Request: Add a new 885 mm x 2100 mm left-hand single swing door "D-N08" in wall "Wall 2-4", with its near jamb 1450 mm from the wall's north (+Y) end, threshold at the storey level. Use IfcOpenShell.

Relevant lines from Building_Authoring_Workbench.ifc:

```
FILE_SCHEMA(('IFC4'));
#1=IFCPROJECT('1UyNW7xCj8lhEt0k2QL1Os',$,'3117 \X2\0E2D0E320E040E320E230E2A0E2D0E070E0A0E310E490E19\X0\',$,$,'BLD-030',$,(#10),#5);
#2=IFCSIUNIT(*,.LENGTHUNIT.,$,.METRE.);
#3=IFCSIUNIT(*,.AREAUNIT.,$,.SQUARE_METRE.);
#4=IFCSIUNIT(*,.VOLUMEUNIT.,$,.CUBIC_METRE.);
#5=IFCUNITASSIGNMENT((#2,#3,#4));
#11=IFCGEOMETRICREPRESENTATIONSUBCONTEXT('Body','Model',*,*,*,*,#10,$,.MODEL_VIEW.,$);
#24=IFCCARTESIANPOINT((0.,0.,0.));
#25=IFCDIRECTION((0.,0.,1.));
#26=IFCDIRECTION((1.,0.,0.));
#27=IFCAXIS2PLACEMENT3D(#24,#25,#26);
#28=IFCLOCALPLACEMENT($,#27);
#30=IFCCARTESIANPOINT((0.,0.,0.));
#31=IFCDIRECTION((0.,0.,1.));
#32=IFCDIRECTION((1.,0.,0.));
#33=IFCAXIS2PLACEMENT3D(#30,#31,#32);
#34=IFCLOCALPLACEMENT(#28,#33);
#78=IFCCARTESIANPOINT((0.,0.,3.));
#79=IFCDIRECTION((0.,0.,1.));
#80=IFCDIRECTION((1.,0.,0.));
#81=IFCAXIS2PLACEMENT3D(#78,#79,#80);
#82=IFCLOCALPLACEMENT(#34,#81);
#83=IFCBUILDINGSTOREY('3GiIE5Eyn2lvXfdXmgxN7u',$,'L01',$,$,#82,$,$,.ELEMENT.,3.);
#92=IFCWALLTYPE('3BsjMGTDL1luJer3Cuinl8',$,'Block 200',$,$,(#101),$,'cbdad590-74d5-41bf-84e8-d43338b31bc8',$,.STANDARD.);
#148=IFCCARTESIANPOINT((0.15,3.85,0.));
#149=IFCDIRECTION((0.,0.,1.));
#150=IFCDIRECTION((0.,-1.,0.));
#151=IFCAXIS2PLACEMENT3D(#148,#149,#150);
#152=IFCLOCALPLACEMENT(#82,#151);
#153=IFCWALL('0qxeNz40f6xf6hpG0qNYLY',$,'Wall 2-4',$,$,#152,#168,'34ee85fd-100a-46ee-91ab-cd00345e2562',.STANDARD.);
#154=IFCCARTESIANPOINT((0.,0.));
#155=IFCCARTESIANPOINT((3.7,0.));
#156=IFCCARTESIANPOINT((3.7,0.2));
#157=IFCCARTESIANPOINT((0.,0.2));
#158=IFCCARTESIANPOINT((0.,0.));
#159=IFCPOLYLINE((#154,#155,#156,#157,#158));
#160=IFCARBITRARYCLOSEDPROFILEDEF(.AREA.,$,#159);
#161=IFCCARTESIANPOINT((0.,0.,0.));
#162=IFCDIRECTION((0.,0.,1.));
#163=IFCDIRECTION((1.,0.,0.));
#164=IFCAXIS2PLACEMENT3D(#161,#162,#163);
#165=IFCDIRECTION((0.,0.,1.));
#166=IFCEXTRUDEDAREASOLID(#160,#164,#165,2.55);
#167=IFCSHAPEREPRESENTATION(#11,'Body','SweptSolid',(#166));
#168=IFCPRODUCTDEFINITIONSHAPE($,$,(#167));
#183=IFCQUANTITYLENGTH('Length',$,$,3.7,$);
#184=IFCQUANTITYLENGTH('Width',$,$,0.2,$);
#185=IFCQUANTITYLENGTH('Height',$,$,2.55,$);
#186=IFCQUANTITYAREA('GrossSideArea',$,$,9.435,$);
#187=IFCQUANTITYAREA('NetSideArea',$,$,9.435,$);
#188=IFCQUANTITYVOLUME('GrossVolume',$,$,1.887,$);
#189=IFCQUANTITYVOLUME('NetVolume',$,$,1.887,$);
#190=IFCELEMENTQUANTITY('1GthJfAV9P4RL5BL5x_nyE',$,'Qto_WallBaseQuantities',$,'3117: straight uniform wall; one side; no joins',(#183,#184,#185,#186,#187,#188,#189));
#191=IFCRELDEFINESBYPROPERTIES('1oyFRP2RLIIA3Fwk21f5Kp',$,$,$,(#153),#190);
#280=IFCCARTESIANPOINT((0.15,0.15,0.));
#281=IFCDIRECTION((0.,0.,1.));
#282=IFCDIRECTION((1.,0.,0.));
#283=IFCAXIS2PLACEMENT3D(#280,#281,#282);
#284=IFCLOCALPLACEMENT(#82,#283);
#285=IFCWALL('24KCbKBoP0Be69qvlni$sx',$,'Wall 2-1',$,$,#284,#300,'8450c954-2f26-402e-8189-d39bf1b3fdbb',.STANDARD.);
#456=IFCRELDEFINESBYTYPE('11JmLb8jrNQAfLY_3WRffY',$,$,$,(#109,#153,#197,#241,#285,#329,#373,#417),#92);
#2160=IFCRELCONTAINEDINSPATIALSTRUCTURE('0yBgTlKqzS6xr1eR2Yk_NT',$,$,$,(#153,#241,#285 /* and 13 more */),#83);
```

```python
import numpy as np
import ifcopenshell
import ifcopenshell.api.feature
import ifcopenshell.api.geometry
import ifcopenshell.api.pset
import ifcopenshell.api.root
import ifcopenshell.api.spatial
import ifcopenshell.geom
import ifcopenshell.util.element
import ifcopenshell.util.placement
import ifcopenshell.util.representation
import ifcopenshell.util.shape
import ifcopenshell.util.unit

model = ifcopenshell.open("Building_Authoring_Workbench.ifc")
unit_scale = ifcopenshell.util.unit.calculate_unit_scale(model)
area_scale = ifcopenshell.util.unit.calculate_unit_scale(model, "AREAUNIT")
volume_scale = ifcopenshell.util.unit.calculate_unit_scale(model, "VOLUMEUNIT")
settings = ifcopenshell.geom.settings()


def volume(element):
    """Net volume in cubic metres, openings subtracted."""
    shape = ifcopenshell.geom.create_shape(settings, element)
    return ifcopenshell.util.shape.get_volume(shape.geometry)


wall = model.by_guid("0qxeNz40f6xf6hpG0qNYLY")
storey = ifcopenshell.util.element.get_container(wall, ifc_class="IfcBuildingStorey")
context = ifcopenshell.util.representation.get_context(model, "Model", "Body", "MODEL_VIEW")
before = volume(wall)

width, height, from_end, sill = 0.885, 2.1, 1.45, 0.0  # metres

# The wall runs along its own X axis, and the end named is its -X end.
wall_shape = ifcopenshell.geom.create_shape(settings, wall)
x, y, z = ifcopenshell.util.shape.get_vertices(wall_shape.geometry).T
start = x.min() + from_end
face, thickness = float(y.min()), float(y.max() - y.min())
wall_matrix = ifcopenshell.util.placement.get_local_placement(wall.ObjectPlacement)
level = ifcopenshell.util.placement.get_local_placement(storey.ObjectPlacement)[2, 3]


def in_wall(x, y):
    """Placement at x, y metres in the wall's axes, at sill height."""
    matrix = wall_matrix.copy()
    matrix[:, 3] = wall_matrix @ np.array([x / unit_scale, y / unit_scale, 0.0, 1.0])
    matrix[2, 3] = level + sill / unit_scale
    return matrix


# Opening: a box that overshoots both wall faces by 50 mm.
opening = ifcopenshell.api.root.create_entity(model, ifc_class="IfcOpeningElement", predefined_type="OPENING")
box = ifcopenshell.api.geometry.add_wall_representation(
    model, context=context, length=width, height=height, thickness=thickness + 0.1
)
ifcopenshell.api.geometry.assign_representation(model, product=opening, representation=box)
ifcopenshell.api.geometry.edit_object_placement(model, product=opening, matrix=in_wall(start, face - 0.05), is_si=False)
ifcopenshell.api.feature.add_feature(model, feature=opening, element=wall)

door = ifcopenshell.api.root.create_entity(model, ifc_class="IfcDoor", name="D-N08", predefined_type="DOOR")
door.OverallWidth, door.OverallHeight = width / unit_scale, height / unit_scale
door.OperationType = "SINGLE_SWING_LEFT"
body = ifcopenshell.api.geometry.add_door_representation(
    model,
    context=context,
    overall_width=door.OverallWidth,
    overall_height=door.OverallHeight,
    operation_type="SINGLE_SWING_LEFT",
    lining_properties={"LiningDepth": thickness / unit_scale, "ThresholdDepth": thickness / unit_scale},
)
ifcopenshell.api.geometry.assign_representation(model, product=door, representation=body)
ifcopenshell.api.spatial.assign_container(model, products=[door], relating_structure=storey)
ifcopenshell.api.feature.add_filling(model, opening=opening, element=door)

# The lining spans the wall, so the door starts at the wall face.
ifcopenshell.api.geometry.edit_object_placement(model, product=door, matrix=in_wall(start, face), is_si=False)

after = volume(wall)

# Update the wall's stored quantities.
qto = model.by_id(ifcopenshell.util.element.get_pset(wall, "Qto_WallBaseQuantities", should_inherit=False)["id"])
ifcopenshell.api.pset.edit_qto(model, qto=qto, properties={
    "NetSideArea": after / thickness / area_scale,
    "NetVolume": after / volume_scale,
})

print(f"wall volume {before:.3f} -> {after:.3f} m3")

model.write("Building_Authoring_Workbench_rev.ifc")
```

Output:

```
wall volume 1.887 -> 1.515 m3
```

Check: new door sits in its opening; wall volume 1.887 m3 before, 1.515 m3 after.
